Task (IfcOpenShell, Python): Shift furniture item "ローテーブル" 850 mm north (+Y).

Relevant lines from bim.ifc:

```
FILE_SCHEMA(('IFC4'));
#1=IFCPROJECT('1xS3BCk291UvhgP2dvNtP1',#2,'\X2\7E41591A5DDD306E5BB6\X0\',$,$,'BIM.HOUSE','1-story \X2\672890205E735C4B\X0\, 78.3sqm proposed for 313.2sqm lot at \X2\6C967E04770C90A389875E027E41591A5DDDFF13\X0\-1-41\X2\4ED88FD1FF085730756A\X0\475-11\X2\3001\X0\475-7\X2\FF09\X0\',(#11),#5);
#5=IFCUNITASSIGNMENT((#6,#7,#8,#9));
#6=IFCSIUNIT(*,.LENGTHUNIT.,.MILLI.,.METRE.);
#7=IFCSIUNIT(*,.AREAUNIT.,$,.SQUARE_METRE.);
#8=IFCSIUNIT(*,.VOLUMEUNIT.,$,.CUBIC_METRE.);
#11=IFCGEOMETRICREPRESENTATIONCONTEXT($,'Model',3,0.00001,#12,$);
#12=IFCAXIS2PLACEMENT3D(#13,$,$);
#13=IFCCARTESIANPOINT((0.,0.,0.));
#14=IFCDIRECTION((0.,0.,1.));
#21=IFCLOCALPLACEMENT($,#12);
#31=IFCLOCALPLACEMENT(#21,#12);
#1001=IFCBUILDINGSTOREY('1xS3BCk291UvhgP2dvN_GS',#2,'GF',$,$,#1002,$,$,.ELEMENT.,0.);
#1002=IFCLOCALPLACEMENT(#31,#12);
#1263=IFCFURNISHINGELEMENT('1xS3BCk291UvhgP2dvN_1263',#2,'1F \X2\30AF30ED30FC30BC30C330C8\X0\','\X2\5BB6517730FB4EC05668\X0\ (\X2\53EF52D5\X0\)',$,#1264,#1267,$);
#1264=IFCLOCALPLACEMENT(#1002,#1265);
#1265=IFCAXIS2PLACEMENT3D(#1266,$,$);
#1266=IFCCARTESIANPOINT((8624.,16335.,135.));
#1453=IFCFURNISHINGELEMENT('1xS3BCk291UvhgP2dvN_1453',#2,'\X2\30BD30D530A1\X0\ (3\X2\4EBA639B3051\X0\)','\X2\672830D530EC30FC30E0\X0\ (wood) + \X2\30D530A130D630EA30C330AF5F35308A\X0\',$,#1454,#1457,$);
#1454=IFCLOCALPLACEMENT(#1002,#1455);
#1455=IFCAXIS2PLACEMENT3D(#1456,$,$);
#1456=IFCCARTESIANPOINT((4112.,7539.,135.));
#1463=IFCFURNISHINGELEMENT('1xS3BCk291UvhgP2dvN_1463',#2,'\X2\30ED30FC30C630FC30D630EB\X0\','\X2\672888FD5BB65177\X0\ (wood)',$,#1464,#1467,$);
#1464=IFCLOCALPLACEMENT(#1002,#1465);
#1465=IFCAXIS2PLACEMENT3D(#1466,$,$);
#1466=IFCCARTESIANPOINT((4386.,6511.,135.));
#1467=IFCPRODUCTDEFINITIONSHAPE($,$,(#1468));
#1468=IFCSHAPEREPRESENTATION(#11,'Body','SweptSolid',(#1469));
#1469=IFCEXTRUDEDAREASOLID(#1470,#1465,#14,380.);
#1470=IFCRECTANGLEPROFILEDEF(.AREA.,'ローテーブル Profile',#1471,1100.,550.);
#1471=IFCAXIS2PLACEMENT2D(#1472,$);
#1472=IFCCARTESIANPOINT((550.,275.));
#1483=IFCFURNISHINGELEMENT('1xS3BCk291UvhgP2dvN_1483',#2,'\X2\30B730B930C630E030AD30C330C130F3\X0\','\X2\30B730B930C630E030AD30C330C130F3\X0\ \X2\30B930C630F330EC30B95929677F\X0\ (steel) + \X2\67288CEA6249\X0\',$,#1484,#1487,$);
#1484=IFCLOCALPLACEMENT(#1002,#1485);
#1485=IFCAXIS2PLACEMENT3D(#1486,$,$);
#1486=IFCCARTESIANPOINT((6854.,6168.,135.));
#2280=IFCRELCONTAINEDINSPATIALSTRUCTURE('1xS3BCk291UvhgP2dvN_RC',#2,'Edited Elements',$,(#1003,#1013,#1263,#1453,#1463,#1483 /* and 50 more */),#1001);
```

```python
import ifcopenshell
import ifcopenshell.api.geometry
import ifcopenshell.util.placement
import ifcopenshell.util.unit

model = ifcopenshell.open("bim.ifc")
unit_scale = ifcopenshell.util.unit.calculate_unit_scale(model)

item = model.by_guid("1xS3BCk291UvhgP2dvN_1463")
matrix = ifcopenshell.util.placement.get_local_placement(item.ObjectPlacement)
matrix[1, 3] += 0.85 / unit_scale
ifcopenshell.api.geometry.edit_object_placement(model, product=item, matrix=matrix, is_si=False)

print(ifcopenshell.util.placement.get_local_placement(item.ObjectPlacement).round(3) + 0.0)

model.write("bim_v2.ifc")
```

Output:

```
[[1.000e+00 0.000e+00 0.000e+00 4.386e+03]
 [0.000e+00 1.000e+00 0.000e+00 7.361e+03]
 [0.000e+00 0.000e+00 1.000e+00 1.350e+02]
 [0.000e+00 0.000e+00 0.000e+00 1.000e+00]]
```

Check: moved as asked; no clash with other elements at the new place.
